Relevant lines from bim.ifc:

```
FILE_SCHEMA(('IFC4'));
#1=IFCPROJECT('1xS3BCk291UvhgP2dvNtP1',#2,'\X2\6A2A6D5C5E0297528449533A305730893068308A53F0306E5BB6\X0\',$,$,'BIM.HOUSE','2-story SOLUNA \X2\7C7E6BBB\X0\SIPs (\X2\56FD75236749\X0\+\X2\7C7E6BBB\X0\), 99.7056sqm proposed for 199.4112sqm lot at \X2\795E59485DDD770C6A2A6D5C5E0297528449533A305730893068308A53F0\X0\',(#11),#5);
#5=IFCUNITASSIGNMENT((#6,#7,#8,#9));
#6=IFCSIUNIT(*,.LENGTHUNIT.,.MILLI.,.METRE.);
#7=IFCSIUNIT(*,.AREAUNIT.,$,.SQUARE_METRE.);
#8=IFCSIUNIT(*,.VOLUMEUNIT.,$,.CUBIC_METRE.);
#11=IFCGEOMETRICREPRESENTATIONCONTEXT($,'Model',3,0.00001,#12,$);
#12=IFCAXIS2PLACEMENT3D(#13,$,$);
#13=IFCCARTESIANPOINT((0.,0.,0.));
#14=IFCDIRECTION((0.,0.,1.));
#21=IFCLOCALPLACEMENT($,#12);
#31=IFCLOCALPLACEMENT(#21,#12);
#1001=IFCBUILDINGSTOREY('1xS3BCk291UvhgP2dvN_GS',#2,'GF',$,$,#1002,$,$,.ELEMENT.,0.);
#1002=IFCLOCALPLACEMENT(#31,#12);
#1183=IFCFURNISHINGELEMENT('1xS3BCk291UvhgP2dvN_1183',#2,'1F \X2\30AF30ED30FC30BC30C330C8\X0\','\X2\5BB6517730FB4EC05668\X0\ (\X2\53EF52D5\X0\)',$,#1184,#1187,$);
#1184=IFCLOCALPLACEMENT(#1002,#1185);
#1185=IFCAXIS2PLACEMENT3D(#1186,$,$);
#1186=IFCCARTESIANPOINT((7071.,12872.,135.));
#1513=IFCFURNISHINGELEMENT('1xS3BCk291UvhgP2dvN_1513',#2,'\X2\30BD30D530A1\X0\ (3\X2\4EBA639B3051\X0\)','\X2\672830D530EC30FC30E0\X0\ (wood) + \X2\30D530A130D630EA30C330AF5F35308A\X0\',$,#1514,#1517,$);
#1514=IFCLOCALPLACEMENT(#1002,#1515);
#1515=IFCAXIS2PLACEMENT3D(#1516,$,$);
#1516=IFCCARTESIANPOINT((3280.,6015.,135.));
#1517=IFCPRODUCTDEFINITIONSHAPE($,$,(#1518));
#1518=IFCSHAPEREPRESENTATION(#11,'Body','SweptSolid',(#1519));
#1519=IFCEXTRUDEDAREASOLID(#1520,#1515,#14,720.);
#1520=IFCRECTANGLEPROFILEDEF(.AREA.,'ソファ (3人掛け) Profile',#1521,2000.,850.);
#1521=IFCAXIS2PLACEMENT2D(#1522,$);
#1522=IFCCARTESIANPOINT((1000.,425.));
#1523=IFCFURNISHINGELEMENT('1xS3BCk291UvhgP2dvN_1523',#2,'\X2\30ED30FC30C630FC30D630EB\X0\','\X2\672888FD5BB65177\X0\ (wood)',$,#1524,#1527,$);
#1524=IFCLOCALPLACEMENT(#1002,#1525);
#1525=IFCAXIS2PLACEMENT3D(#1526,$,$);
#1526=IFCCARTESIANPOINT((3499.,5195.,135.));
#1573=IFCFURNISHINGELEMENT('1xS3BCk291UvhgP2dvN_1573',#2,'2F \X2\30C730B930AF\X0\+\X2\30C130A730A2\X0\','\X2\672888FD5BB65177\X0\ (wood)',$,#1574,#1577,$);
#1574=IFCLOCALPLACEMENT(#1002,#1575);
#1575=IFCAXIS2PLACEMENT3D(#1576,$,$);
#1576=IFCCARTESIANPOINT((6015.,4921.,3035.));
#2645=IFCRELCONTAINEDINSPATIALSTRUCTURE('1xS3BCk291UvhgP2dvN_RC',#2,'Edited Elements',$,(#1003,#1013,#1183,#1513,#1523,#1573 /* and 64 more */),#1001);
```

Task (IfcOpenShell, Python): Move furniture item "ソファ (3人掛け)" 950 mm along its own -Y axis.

```python
import ifcopenshell
import ifcopenshell.api.geometry
import ifcopenshell.util.placement
import ifcopenshell.util.unit

model = ifcopenshell.open("bim.ifc")
unit_scale = ifcopenshell.util.unit.calculate_unit_scale(model)

item = model.by_guid("1xS3BCk291UvhgP2dvN_1513")
matrix = ifcopenshell.util.placement.get_local_placement(item.ObjectPlacement)
matrix[:3, 3] -= matrix[:3, 1] * 0.95 / unit_scale
ifcopenshell.api.geometry.edit_object_placement(model, product=item, matrix=matrix, is_si=False)

print(ifcopenshell.util.placement.get_local_placement(item.ObjectPlacement).round(3) + 0.0)

model.write("bim_v2.ifc")
```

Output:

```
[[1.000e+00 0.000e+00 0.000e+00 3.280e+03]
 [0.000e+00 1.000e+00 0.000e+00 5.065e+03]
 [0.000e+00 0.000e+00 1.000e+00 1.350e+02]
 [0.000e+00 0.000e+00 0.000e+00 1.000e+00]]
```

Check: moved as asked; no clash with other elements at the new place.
